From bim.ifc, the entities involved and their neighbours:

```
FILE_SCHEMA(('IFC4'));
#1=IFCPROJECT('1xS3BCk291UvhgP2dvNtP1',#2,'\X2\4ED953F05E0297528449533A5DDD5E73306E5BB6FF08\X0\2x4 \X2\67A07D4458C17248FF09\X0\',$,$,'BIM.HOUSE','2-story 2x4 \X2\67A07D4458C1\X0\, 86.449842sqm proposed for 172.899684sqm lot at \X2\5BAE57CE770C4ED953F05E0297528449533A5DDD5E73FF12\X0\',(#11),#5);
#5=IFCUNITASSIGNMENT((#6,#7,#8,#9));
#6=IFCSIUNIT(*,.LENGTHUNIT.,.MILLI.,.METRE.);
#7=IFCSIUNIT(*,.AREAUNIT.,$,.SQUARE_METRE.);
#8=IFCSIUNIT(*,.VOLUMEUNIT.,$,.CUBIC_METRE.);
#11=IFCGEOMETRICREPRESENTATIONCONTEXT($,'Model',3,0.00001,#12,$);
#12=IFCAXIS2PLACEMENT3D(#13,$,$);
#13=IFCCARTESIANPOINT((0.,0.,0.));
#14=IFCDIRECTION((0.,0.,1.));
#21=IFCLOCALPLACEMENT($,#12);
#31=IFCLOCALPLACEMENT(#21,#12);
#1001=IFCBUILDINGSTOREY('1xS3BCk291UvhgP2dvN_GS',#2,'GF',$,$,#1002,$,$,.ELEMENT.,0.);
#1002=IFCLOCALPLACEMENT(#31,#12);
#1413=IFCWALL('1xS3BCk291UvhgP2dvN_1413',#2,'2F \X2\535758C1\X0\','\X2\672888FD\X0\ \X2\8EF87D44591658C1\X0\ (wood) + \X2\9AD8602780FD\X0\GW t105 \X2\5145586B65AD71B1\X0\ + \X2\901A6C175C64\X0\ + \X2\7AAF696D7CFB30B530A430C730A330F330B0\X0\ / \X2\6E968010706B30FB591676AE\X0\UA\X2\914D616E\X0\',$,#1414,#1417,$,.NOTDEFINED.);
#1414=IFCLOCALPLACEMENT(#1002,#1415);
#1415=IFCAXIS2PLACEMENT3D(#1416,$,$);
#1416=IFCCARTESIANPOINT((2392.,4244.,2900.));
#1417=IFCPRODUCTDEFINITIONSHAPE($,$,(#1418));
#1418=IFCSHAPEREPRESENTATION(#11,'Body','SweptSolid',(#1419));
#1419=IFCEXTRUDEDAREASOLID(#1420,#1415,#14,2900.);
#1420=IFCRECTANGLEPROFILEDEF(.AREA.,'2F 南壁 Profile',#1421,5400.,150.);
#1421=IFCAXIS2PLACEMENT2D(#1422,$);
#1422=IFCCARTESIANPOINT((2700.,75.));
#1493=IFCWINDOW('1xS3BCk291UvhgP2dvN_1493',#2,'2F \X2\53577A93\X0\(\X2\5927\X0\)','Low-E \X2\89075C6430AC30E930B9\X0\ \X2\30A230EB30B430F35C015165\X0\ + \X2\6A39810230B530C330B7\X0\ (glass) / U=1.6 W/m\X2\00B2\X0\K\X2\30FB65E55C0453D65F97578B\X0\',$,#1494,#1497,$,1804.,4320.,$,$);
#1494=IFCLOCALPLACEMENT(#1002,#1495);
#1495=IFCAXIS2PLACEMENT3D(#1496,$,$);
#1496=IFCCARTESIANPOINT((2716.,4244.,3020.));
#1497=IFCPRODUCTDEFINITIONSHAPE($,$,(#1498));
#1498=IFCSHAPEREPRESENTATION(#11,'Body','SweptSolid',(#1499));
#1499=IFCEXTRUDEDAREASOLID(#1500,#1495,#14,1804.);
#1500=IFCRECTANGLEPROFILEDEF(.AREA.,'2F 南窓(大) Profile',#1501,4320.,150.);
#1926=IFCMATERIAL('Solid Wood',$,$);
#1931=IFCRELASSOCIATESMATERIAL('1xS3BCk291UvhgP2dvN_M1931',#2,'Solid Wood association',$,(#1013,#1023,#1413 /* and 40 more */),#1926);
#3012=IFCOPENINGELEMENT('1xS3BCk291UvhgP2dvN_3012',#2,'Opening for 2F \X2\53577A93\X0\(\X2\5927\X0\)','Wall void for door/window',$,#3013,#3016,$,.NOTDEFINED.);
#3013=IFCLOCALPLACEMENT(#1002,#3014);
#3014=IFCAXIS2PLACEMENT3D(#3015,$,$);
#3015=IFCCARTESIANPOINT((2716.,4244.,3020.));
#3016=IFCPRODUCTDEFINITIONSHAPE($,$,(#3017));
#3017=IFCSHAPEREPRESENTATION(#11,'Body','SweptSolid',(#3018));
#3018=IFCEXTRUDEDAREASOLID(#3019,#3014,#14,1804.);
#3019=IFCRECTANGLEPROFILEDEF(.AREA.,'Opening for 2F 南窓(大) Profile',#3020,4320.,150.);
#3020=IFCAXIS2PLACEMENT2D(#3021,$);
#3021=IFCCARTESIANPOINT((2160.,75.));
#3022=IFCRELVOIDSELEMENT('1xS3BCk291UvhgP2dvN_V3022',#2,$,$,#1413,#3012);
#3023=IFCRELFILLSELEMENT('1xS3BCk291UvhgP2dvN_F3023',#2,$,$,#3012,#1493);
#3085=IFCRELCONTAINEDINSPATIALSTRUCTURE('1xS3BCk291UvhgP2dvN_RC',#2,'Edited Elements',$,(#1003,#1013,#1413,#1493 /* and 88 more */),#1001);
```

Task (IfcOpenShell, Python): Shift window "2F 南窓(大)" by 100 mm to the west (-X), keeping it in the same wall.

```python
import ifcopenshell
import ifcopenshell.api.geometry
import ifcopenshell.util.placement
import ifcopenshell.util.unit

model = ifcopenshell.open("bim.ifc")
unit_scale = ifcopenshell.util.unit.calculate_unit_scale(model)

window = model.by_id(1493)
opening = window.FillsVoids[0].RelatingOpeningElement
wall = opening.VoidsElements[0].RelatingBuildingElement

wall_matrix = ifcopenshell.util.placement.get_local_placement(wall.ObjectPlacement)
shift = wall_matrix[:3, 0] * -0.1 / unit_scale
before = ifcopenshell.util.placement.get_local_placement(window.ObjectPlacement)[:3, 3].copy()

# The window is not placed relative to its opening, so move both.
for product in (opening, window):
    matrix = ifcopenshell.util.placement.get_local_placement(product.ObjectPlacement)
    matrix[:3, 3] += shift
    ifcopenshell.api.geometry.edit_object_placement(model, product=product, matrix=matrix, is_si=False)

after = ifcopenshell.util.placement.get_local_placement(window.ObjectPlacement)[:3, 3]
print("window moved by", (after - before).round(3) + 0.0)

model.write("bim_edited.ifc")
```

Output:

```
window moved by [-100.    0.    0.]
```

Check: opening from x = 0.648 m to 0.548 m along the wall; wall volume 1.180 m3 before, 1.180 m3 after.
